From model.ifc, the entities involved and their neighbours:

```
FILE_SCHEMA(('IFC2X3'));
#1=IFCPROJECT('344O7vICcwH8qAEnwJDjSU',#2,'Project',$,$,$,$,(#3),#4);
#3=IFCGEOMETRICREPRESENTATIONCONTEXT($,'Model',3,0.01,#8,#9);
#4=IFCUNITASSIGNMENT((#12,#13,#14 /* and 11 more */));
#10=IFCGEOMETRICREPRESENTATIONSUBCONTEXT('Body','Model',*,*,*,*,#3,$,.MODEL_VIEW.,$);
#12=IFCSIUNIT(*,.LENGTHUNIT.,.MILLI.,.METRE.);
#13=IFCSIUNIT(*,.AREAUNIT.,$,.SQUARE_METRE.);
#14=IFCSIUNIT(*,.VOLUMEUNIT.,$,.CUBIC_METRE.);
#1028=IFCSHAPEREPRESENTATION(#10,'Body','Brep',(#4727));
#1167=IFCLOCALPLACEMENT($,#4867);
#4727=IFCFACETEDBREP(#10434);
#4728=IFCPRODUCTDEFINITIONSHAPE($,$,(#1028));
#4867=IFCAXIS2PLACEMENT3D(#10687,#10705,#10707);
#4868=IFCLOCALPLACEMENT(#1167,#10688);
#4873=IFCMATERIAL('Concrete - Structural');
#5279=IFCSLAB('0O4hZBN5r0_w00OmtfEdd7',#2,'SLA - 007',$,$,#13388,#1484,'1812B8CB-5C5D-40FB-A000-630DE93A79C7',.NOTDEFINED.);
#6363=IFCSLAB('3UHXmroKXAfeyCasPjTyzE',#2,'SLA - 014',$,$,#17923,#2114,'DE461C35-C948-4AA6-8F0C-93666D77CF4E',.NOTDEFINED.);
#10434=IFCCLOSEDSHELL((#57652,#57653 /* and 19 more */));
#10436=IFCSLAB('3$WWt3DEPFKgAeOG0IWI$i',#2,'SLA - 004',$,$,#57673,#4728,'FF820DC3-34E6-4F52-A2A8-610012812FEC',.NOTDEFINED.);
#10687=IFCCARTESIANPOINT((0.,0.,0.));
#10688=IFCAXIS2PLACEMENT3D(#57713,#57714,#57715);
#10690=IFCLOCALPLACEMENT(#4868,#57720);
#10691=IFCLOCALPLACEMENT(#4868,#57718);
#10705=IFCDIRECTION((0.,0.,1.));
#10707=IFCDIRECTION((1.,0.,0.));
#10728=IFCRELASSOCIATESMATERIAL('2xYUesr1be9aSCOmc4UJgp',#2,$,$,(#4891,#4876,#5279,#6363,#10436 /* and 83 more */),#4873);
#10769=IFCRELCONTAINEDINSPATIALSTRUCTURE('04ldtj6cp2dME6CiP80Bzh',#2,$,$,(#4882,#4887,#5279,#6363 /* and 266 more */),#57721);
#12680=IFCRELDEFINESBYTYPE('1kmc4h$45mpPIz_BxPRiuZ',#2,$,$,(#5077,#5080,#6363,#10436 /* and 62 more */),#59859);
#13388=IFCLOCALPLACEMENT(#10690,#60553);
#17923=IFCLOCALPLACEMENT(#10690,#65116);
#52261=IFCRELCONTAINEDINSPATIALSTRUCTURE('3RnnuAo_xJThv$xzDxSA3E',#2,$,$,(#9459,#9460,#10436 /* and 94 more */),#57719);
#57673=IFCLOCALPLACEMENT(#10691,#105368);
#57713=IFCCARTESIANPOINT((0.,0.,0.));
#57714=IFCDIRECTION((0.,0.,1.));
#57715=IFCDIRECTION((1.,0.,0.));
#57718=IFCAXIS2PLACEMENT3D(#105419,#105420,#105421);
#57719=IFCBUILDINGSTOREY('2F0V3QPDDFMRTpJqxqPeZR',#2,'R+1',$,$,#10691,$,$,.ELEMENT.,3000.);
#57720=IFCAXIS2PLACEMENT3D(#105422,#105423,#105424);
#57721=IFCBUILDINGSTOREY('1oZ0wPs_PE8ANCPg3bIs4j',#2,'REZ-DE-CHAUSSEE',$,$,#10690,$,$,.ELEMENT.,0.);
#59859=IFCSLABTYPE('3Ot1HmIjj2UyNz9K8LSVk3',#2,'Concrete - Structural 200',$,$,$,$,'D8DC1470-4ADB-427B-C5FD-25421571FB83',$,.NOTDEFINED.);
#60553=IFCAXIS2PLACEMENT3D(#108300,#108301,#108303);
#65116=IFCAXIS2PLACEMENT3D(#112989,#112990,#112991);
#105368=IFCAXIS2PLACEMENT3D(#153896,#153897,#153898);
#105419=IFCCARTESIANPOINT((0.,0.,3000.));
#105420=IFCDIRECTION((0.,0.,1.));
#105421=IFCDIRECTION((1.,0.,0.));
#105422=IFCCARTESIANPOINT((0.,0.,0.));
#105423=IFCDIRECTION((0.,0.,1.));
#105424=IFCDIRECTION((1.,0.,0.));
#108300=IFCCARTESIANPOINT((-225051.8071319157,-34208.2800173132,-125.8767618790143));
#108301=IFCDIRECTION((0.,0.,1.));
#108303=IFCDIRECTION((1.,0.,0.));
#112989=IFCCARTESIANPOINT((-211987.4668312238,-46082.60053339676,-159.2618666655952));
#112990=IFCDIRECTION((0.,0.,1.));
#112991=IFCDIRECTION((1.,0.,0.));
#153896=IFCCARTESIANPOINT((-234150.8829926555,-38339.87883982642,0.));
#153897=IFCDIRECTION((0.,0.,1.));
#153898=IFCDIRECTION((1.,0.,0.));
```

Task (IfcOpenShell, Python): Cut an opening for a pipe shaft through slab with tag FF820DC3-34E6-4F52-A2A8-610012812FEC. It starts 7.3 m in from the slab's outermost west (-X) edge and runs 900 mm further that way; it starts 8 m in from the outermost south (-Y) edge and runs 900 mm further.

```python
import numpy as np
import ifcopenshell
import ifcopenshell.api.feature
import ifcopenshell.api.geometry
import ifcopenshell.api.root
import ifcopenshell.geom
import ifcopenshell.util.placement
import ifcopenshell.util.representation
import ifcopenshell.util.shape
import ifcopenshell.util.unit

model = ifcopenshell.open("model.ifc")
unit_scale = ifcopenshell.util.unit.calculate_unit_scale(model)
settings = ifcopenshell.geom.settings()


def volume(element):
    """Net volume in cubic metres, openings subtracted."""
    shape = ifcopenshell.geom.create_shape(settings, element)
    return ifcopenshell.util.shape.get_volume(shape.geometry)


slab = model.by_id(10436)
before = volume(slab)

# Extent in the slab's own axes, in metres. The edges named are its -X and -Y sides.
slab_shape = ifcopenshell.geom.create_shape(settings, slab)
vertices = ifcopenshell.util.shape.get_vertices(slab_shape.geometry)
x_min, y_min, bottom = vertices.min(axis=0)
top = vertices[:, 2].max()

opening = ifcopenshell.api.root.create_entity(model, ifc_class="IfcOpeningElement", name="Pipe shaft opening")
context = ifcopenshell.util.representation.get_context(model, "Model", "Body", "MODEL_VIEW")
width, depth = 0.9, 0.9
outline = [(0.0, 0.0), (width, 0.0), (width, depth), (0.0, depth), (0.0, 0.0)]
# Overshoot both faces by 50 mm so the cut is clean.
shape = ifcopenshell.api.geometry.add_slab_representation(
    model, context=context, depth=top - bottom + 0.1, polyline=outline
)
ifcopenshell.api.geometry.assign_representation(model, product=opening, representation=shape)

matrix = ifcopenshell.util.placement.get_local_placement(slab.ObjectPlacement)
matrix[:, 3] = matrix @ np.append(np.array([x_min + 7.3, y_min + 8, bottom - 0.05]) / unit_scale, 1.0)
ifcopenshell.api.geometry.edit_object_placement(model, product=opening, matrix=matrix, is_si=False)
ifcopenshell.api.feature.add_feature(model, feature=opening, element=slab)

after = volume(slab)

print(f"slab volume {before:.3f} -> {after:.3f} m3")

model.write("model_updated.ifc")
```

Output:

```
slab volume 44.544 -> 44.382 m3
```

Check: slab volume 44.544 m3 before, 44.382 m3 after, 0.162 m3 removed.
